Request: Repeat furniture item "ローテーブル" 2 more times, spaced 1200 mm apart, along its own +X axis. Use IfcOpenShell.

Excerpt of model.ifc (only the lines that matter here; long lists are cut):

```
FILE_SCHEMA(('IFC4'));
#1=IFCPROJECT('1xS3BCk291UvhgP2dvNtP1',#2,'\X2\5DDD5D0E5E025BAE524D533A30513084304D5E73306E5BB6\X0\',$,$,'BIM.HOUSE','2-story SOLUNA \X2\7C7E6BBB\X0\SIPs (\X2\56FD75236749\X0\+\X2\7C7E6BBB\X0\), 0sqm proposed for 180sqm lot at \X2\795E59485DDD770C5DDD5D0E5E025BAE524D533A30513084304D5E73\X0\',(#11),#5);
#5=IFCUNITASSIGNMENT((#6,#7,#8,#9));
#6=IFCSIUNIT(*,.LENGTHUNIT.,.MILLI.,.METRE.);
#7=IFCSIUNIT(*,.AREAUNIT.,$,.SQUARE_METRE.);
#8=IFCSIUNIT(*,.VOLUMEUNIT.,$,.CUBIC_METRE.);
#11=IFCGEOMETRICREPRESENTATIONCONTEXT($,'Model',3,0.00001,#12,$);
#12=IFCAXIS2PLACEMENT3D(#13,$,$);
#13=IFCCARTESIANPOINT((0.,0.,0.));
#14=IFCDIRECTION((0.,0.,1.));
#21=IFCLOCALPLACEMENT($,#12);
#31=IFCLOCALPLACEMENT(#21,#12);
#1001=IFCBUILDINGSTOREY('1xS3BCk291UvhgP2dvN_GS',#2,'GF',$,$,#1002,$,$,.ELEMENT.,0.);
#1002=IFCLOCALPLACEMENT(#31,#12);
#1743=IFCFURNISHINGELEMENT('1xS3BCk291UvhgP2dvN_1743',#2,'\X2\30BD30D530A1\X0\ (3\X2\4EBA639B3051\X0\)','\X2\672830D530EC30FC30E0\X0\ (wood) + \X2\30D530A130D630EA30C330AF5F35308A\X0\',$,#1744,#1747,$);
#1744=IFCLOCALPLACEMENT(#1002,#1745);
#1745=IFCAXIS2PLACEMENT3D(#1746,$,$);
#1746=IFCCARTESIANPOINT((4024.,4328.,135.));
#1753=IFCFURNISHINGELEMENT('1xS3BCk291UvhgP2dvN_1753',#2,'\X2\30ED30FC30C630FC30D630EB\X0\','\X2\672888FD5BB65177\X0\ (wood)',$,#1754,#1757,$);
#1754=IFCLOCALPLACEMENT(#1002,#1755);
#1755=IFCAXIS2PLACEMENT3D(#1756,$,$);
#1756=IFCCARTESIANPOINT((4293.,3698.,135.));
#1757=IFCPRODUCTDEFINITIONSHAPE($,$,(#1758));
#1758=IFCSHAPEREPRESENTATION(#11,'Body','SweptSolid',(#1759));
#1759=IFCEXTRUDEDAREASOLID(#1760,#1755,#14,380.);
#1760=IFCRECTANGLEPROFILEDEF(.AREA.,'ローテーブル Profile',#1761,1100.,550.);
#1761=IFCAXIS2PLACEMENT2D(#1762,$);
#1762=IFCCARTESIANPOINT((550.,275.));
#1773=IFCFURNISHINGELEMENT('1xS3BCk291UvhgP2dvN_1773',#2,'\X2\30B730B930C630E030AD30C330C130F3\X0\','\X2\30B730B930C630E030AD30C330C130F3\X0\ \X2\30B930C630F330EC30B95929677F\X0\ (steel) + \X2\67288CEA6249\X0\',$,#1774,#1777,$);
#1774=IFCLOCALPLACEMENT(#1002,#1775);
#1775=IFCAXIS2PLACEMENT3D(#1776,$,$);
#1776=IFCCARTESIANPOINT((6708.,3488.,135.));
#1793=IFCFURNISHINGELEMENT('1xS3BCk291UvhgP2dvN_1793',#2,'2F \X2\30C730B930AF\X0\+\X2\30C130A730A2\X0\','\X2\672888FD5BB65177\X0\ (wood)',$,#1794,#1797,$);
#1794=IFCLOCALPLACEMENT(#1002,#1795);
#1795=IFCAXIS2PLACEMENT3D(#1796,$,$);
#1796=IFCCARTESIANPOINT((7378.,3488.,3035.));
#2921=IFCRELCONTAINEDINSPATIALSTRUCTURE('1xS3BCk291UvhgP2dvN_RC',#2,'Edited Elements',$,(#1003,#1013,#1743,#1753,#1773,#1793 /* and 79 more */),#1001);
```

```python
import ifcopenshell
import ifcopenshell.api.geometry
import ifcopenshell.api.root
import ifcopenshell.util.element
import ifcopenshell.util.placement

model = ifcopenshell.open("model.ifc")


def reuse_history(source, copy):
    """copy_class also copies each property set's owner history, people and application; keep the originals."""
    for rel in copy.IsDefinedBy:
        if rel.is_a("IfcRelDefinesByProperties") and (history := rel.RelatingPropertyDefinition.OwnerHistory):
            rel.RelatingPropertyDefinition.OwnerHistory = source.OwnerHistory
            ifcopenshell.util.element.remove_deep2(model, history)


source = model.by_guid("1xS3BCk291UvhgP2dvN_1753")
base = ifcopenshell.util.placement.get_local_placement(source.ObjectPlacement)
step = base[:3, 0] * 1200.0

for i in range(1, 3):
    copy = ifcopenshell.api.root.copy_class(model, product=source)
    copy.Representation = ifcopenshell.util.element.copy_deep(
        model, source.Representation, exclude=["IfcGeometricRepresentationContext", "IfcRepresentationMap"]
    )
    reuse_history(source, copy)
    matrix = base.copy()
    matrix[:3, 3] += i * step
    print("added at", matrix[:3, 3].round(3) + 0.0)
    ifcopenshell.api.geometry.edit_object_placement(model, product=copy, matrix=matrix, is_si=False)

model.write("model-out.ifc")
```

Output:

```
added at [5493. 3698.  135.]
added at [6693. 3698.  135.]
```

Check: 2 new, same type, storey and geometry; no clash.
